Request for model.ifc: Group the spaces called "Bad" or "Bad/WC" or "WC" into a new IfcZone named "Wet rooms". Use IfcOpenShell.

First a look at what the model holds.

```python
import ifcopenshell

model = ifcopenshell.open("model.ifc")
print(model.schema)
seen = {}
for space in model.by_type("IfcSpace"):
    seen[space.LongName] = seen.get(space.LongName, 0) + 1
for name, count in sorted(seen.items(), key=str):
    print(count, "x", name)
print("zones:", [z.Name for z in model.by_type("IfcZone")][:20])
```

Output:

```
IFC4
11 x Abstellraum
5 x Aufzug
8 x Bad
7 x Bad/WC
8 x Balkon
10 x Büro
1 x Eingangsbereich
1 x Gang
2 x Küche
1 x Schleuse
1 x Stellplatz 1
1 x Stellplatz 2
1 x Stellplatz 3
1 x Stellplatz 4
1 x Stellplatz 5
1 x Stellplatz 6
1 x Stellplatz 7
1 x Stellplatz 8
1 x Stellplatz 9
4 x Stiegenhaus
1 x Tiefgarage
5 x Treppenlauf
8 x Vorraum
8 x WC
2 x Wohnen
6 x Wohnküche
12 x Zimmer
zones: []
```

```python
import ifcopenshell
import ifcopenshell.api.group
import ifcopenshell.api.root

model = ifcopenshell.open("model.ifc")

names = {"Bad", "Bad/WC", "WC"}
spaces = [s for s in model.by_type("IfcSpace") if s.LongName in names]

zone = ifcopenshell.api.root.create_entity(model, ifc_class="IfcZone", name="Wet rooms")
ifcopenshell.api.group.assign_group(model, products=spaces, group=zone)
print(len(spaces), "spaces in", zone.Name)

model.write("model_v2.ifc")
```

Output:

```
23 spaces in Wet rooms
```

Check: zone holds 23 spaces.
